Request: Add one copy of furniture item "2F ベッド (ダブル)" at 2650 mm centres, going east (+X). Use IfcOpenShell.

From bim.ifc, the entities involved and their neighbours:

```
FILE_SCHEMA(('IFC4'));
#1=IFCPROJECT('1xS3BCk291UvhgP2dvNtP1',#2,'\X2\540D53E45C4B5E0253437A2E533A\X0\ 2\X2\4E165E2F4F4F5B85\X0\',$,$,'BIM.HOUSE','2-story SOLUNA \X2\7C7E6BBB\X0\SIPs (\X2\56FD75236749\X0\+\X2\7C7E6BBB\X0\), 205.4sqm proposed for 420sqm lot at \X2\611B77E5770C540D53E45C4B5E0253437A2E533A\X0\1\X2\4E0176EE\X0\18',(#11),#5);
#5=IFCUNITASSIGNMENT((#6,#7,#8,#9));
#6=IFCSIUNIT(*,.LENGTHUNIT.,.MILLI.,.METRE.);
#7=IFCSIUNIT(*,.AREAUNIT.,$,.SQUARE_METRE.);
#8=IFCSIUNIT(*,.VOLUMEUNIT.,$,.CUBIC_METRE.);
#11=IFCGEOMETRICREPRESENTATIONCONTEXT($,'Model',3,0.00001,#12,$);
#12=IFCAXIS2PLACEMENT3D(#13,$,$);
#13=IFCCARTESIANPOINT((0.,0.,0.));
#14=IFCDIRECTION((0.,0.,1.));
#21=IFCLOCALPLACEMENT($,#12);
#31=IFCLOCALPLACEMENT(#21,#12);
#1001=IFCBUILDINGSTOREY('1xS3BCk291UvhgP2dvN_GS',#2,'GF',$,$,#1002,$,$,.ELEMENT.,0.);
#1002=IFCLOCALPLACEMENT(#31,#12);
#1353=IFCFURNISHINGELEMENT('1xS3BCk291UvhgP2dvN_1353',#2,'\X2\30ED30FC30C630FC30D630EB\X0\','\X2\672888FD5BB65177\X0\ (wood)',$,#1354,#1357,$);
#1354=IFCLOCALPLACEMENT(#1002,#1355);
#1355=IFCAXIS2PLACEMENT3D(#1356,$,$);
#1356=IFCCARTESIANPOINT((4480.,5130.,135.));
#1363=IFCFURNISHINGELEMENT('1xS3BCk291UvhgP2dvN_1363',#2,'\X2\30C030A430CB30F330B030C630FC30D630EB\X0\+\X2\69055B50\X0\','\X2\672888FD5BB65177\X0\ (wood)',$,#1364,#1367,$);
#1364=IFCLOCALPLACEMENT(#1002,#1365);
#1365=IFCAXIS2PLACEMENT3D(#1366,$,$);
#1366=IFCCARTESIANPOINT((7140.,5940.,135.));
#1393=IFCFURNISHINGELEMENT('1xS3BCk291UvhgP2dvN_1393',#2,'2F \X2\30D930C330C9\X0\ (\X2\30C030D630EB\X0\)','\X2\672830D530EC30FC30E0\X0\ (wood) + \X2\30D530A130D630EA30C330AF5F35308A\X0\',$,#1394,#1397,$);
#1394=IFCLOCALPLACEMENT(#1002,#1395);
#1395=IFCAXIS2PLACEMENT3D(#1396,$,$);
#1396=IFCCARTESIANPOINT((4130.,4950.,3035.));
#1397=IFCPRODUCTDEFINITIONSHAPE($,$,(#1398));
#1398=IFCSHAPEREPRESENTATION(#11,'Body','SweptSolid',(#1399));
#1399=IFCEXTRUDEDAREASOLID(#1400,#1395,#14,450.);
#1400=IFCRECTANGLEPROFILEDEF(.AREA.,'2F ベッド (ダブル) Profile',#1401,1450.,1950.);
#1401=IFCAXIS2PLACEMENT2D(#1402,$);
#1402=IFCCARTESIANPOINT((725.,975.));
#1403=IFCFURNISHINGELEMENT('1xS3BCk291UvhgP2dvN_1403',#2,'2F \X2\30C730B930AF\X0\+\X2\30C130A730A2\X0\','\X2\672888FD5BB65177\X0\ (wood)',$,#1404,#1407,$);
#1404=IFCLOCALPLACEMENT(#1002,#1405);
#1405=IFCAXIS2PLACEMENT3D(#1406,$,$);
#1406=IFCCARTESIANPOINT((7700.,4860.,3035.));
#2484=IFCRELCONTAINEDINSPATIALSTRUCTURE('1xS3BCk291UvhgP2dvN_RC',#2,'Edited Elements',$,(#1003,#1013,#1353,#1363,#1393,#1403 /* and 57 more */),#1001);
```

```python
import numpy as np
import ifcopenshell
import ifcopenshell.api.geometry
import ifcopenshell.api.root
import ifcopenshell.util.element
import ifcopenshell.util.placement

model = ifcopenshell.open("bim.ifc")


def reuse_history(source, copy):
    """copy_class also copies each property set's owner history, people and application; keep the originals."""
    for rel in copy.IsDefinedBy:
        if rel.is_a("IfcRelDefinesByProperties") and (history := rel.RelatingPropertyDefinition.OwnerHistory):
            rel.RelatingPropertyDefinition.OwnerHistory = source.OwnerHistory
            ifcopenshell.util.element.remove_deep2(model, history)


source = model.by_guid("1xS3BCk291UvhgP2dvN_1393")
base = ifcopenshell.util.placement.get_local_placement(source.ObjectPlacement)
step = np.array([1.0, 0.0, 0.0]) * 2650.0

for i in range(1, 2):
    copy = ifcopenshell.api.root.copy_class(model, product=source)
    copy.Representation = ifcopenshell.util.element.copy_deep(
        model, source.Representation, exclude=["IfcGeometricRepresentationContext", "IfcRepresentationMap"]
    )
    reuse_history(source, copy)
    matrix = base.copy()
    matrix[:3, 3] += i * step
    print("added at", matrix[:3, 3].round(3) + 0.0)
    ifcopenshell.api.geometry.edit_object_placement(model, product=copy, matrix=matrix, is_si=False)

model.write("bim_updated.ifc")
```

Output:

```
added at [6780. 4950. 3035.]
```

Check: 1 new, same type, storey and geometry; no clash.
